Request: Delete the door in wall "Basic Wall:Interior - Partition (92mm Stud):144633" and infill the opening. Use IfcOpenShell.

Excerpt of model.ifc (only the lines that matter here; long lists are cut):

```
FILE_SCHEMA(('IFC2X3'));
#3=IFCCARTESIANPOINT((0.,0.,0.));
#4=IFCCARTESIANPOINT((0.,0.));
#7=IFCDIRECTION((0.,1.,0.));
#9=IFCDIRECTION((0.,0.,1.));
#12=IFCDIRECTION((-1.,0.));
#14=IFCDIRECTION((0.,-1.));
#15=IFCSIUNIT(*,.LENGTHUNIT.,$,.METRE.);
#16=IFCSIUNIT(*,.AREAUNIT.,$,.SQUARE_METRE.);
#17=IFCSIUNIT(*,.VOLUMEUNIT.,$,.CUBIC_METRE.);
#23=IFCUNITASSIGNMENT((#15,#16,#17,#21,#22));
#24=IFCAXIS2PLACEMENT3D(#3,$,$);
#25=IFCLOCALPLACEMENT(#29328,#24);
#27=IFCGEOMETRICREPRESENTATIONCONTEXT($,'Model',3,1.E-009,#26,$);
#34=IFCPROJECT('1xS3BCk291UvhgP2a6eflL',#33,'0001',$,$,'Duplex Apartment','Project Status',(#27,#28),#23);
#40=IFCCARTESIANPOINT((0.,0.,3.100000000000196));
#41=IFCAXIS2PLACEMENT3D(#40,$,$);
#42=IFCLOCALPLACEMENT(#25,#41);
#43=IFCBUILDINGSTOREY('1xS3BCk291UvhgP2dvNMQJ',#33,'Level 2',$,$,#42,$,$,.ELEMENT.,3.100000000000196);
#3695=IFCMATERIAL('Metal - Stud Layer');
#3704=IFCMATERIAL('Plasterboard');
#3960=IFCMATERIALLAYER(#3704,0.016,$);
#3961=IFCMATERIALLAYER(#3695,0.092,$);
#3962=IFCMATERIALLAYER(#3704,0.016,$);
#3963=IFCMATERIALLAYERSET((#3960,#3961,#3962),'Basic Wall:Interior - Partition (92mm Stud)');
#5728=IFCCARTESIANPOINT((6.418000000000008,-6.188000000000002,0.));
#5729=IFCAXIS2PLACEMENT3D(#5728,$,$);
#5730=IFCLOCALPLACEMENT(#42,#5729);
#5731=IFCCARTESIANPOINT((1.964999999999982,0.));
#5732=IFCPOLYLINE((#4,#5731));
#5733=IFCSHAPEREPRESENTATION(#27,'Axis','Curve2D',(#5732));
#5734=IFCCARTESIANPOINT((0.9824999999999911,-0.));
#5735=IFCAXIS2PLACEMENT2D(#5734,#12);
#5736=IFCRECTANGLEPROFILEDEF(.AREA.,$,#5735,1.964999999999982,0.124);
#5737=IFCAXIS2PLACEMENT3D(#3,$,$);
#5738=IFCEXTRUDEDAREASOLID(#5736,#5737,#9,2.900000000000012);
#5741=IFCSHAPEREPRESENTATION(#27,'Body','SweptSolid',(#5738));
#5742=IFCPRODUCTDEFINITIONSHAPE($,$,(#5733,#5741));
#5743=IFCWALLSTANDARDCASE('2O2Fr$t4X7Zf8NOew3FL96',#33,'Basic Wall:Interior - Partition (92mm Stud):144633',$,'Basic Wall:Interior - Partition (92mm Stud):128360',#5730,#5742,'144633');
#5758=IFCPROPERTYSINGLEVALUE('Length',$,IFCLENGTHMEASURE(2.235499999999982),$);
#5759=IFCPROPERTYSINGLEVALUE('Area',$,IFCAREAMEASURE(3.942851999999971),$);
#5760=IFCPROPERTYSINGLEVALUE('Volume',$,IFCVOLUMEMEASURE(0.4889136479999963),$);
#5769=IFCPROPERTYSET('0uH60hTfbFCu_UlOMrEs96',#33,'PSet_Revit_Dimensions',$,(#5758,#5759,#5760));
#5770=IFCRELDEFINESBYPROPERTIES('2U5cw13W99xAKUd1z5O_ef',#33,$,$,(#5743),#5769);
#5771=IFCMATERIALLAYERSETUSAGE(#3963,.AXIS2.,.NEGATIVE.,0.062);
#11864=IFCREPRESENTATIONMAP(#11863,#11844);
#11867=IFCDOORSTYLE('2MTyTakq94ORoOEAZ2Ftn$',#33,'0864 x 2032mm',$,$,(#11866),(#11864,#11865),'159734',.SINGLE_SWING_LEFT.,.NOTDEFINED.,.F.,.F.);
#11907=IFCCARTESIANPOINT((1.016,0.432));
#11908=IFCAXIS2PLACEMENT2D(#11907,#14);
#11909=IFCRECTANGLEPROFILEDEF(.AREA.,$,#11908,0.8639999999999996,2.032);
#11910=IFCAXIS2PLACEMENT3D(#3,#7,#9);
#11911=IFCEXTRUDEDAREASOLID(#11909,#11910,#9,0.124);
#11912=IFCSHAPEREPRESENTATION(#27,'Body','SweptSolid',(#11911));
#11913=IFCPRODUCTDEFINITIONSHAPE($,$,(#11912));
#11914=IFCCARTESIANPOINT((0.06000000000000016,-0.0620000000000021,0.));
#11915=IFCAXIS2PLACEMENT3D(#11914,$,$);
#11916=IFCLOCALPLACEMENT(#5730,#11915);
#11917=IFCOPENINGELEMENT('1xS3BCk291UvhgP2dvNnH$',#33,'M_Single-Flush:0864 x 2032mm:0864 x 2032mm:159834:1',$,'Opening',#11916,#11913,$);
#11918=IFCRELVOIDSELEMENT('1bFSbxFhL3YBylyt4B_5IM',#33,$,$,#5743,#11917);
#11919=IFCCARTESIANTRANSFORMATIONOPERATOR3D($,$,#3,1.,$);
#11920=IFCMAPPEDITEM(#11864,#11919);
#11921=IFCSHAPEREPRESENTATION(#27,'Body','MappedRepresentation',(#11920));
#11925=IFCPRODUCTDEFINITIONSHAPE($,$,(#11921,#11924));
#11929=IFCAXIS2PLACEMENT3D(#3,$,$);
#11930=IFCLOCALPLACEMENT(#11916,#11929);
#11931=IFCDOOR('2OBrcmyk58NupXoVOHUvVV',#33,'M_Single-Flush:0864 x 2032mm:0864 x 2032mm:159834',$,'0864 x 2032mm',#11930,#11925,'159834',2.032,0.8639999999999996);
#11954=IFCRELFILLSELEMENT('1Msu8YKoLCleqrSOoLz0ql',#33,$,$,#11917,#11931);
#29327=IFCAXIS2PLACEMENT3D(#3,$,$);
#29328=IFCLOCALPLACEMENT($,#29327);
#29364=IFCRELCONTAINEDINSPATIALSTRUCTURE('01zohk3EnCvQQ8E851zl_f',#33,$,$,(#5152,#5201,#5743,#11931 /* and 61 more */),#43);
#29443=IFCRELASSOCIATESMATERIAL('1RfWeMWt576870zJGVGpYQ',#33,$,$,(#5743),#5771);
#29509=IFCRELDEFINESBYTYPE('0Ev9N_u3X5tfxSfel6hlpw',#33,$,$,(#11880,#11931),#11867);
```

```python
import ifcopenshell
import ifcopenshell.api.feature
import ifcopenshell.api.pset
import ifcopenshell.api.root
import ifcopenshell.geom
import ifcopenshell.util.element
import ifcopenshell.util.shape
import ifcopenshell.util.unit

model = ifcopenshell.open("model.ifc")
area_scale = ifcopenshell.util.unit.calculate_unit_scale(model, "AREAUNIT")
volume_scale = ifcopenshell.util.unit.calculate_unit_scale(model, "VOLUMEUNIT")
settings = ifcopenshell.geom.settings()


def volume(element):
    """Net volume in cubic metres, openings subtracted."""
    shape = ifcopenshell.geom.create_shape(settings, element)
    return ifcopenshell.util.shape.get_volume(shape.geometry)


door = model.by_guid("2OBrcmyk58NupXoVOHUvVV")
opening = door.FillsVoids[0].RelatingOpeningElement
wall = opening.VoidsElements[0].RelatingBuildingElement
before = volume(wall)

ifcopenshell.api.root.remove_product(model, product=door)
ifcopenshell.api.feature.remove_feature(model, feature=opening)

after = volume(wall)
thickness = 0.124  # wall thickness in metres

# Update the wall's stored quantities.
pset = model.by_id(ifcopenshell.util.element.get_pset(wall, "PSet_Revit_Dimensions", should_inherit=False)["id"])
ifcopenshell.api.pset.edit_pset(model, pset=pset, properties={
    "Area": model.create_entity("IfcAreaMeasure", after / thickness / area_scale),
    "Volume": model.create_entity("IfcVolumeMeasure", after / volume_scale),
})

print(f"wall volume {before:.3f} -> {after:.3f} m3")

model.write("model_edited.ifc")
```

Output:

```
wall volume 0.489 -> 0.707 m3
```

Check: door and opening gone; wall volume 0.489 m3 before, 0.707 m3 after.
